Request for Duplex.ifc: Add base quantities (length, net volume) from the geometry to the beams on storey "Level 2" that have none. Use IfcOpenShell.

First a look at what the model holds.

```python
import ifcopenshell
import ifcopenshell.util.element
import ifcopenshell.util.unit

model = ifcopenshell.open("Duplex.ifc")
print(model.schema)
for unit_type in ("LENGTHUNIT", "AREAUNIT", "VOLUMEUNIT"):
    print(unit_type, ifcopenshell.util.unit.calculate_unit_scale(model, unit_type))
storey = next(s for s in model.by_type("IfcBuildingStorey") if s.Name == "Level 2")
beams = [e for e in ifcopenshell.util.element.get_decomposition(storey) if e.is_a("IfcBeam")]
for e in sorted(beams, key=lambda e: e.id()):
    print(e.id(), e.is_a(), e.Name, list(ifcopenshell.util.element.get_psets(e, qtos_only=True)), sep=" | ")
```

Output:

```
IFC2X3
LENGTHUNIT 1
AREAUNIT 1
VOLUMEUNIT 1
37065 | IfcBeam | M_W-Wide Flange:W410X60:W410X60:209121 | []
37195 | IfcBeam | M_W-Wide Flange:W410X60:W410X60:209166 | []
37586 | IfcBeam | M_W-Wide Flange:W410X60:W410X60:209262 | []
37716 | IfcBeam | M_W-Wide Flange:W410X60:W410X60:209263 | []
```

```python
import ifcopenshell
import ifcopenshell.api.pset
import ifcopenshell.geom
import ifcopenshell.util.element
import ifcopenshell.util.shape
import ifcopenshell.util.unit

model = ifcopenshell.open("Duplex.ifc")
unit_scale = ifcopenshell.util.unit.calculate_unit_scale(model)
volume_scale = ifcopenshell.util.unit.calculate_unit_scale(model, "VOLUMEUNIT")
settings = ifcopenshell.geom.settings()

storey = next(s for s in model.by_type("IfcBuildingStorey") if s.Name == "Level 2")
beams = [e for e in ifcopenshell.util.element.get_decomposition(storey) if e.is_a("IfcBeam")]

for e in sorted(beams, key=lambda e: e.id()):
    if ifcopenshell.util.element.get_psets(e, qtos_only=True, should_inherit=False):
        continue
    # Geometry comes back in metres, in the element's own axes.
    shape = ifcopenshell.geom.create_shape(settings, e)
    values = {
        "Length": ifcopenshell.util.shape.get_max_xyz(shape.geometry) / unit_scale,
        "NetVolume": ifcopenshell.util.shape.get_volume(shape.geometry) / volume_scale,
    }
    qto = ifcopenshell.api.pset.add_qto(model, product=e, name="BaseQuantities")
    ifcopenshell.api.pset.edit_qto(model, qto=qto, properties=values)
    print(e.id(), {k: round(v, 3) for k, v in values.items()})

model.write("Duplex_edited.ifc")
```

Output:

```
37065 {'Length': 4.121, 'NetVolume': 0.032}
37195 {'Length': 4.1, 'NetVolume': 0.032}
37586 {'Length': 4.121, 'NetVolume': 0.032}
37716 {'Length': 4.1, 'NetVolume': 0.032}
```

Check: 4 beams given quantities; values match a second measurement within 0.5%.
